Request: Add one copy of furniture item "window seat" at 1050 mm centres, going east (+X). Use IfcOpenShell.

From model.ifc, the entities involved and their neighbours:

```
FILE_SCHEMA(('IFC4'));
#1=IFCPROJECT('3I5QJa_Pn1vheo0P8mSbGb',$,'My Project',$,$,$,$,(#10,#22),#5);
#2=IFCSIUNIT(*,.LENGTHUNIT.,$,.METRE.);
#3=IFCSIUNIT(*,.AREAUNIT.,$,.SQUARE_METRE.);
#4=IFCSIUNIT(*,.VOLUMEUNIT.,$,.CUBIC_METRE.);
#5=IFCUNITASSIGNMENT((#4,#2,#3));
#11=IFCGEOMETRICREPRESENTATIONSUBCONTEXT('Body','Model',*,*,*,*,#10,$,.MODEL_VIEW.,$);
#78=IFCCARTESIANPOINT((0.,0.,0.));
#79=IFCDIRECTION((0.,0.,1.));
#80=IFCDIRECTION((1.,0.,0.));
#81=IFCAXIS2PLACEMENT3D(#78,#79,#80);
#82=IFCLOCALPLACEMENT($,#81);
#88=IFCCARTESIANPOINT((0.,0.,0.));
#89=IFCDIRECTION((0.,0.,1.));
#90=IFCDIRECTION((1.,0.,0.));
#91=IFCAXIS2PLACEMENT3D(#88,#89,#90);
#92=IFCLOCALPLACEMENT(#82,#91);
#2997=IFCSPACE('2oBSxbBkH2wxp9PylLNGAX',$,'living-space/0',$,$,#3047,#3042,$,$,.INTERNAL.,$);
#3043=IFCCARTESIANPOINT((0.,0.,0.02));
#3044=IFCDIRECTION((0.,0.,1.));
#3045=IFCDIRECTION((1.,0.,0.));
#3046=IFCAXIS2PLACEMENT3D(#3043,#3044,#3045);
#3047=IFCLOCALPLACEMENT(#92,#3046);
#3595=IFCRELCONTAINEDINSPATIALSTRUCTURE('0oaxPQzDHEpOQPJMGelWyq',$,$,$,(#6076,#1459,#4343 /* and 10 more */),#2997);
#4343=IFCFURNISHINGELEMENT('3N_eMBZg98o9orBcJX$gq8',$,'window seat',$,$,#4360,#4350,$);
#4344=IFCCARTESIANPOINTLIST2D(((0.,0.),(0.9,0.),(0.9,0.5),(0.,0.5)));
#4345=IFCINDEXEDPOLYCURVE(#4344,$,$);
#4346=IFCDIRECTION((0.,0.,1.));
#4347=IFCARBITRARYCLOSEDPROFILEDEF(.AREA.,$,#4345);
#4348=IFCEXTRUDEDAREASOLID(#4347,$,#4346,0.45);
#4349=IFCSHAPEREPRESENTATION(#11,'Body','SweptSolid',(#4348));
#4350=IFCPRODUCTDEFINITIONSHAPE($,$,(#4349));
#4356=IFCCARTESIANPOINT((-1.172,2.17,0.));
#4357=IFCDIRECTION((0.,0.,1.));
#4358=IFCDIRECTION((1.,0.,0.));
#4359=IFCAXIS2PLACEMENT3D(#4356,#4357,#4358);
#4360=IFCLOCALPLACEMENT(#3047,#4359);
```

```python
import numpy as np
import ifcopenshell
import ifcopenshell.api.geometry
import ifcopenshell.api.root
import ifcopenshell.util.element
import ifcopenshell.util.placement
import ifcopenshell.util.unit

model = ifcopenshell.open("model.ifc")
unit_scale = ifcopenshell.util.unit.calculate_unit_scale(model)

source = model.by_guid("3N_eMBZg98o9orBcJX$gq8")
base = ifcopenshell.util.placement.get_local_placement(source.ObjectPlacement)
step = np.array([1.0, 0.0, 0.0]) * 1.05 / unit_scale

for i in range(1, 2):
    copy = ifcopenshell.api.root.copy_class(model, product=source)
    copy.Representation = ifcopenshell.util.element.copy_deep(
        model, source.Representation, exclude=["IfcGeometricRepresentationContext", "IfcRepresentationMap"]
    )
    matrix = base.copy()
    matrix[:3, 3] += i * step
    print("added at", matrix[:3, 3].round(3) + 0.0)
    ifcopenshell.api.geometry.edit_object_placement(model, product=copy, matrix=matrix, is_si=False)

model.write("model_edited.ifc")
```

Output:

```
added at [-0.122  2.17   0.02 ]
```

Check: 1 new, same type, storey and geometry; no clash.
